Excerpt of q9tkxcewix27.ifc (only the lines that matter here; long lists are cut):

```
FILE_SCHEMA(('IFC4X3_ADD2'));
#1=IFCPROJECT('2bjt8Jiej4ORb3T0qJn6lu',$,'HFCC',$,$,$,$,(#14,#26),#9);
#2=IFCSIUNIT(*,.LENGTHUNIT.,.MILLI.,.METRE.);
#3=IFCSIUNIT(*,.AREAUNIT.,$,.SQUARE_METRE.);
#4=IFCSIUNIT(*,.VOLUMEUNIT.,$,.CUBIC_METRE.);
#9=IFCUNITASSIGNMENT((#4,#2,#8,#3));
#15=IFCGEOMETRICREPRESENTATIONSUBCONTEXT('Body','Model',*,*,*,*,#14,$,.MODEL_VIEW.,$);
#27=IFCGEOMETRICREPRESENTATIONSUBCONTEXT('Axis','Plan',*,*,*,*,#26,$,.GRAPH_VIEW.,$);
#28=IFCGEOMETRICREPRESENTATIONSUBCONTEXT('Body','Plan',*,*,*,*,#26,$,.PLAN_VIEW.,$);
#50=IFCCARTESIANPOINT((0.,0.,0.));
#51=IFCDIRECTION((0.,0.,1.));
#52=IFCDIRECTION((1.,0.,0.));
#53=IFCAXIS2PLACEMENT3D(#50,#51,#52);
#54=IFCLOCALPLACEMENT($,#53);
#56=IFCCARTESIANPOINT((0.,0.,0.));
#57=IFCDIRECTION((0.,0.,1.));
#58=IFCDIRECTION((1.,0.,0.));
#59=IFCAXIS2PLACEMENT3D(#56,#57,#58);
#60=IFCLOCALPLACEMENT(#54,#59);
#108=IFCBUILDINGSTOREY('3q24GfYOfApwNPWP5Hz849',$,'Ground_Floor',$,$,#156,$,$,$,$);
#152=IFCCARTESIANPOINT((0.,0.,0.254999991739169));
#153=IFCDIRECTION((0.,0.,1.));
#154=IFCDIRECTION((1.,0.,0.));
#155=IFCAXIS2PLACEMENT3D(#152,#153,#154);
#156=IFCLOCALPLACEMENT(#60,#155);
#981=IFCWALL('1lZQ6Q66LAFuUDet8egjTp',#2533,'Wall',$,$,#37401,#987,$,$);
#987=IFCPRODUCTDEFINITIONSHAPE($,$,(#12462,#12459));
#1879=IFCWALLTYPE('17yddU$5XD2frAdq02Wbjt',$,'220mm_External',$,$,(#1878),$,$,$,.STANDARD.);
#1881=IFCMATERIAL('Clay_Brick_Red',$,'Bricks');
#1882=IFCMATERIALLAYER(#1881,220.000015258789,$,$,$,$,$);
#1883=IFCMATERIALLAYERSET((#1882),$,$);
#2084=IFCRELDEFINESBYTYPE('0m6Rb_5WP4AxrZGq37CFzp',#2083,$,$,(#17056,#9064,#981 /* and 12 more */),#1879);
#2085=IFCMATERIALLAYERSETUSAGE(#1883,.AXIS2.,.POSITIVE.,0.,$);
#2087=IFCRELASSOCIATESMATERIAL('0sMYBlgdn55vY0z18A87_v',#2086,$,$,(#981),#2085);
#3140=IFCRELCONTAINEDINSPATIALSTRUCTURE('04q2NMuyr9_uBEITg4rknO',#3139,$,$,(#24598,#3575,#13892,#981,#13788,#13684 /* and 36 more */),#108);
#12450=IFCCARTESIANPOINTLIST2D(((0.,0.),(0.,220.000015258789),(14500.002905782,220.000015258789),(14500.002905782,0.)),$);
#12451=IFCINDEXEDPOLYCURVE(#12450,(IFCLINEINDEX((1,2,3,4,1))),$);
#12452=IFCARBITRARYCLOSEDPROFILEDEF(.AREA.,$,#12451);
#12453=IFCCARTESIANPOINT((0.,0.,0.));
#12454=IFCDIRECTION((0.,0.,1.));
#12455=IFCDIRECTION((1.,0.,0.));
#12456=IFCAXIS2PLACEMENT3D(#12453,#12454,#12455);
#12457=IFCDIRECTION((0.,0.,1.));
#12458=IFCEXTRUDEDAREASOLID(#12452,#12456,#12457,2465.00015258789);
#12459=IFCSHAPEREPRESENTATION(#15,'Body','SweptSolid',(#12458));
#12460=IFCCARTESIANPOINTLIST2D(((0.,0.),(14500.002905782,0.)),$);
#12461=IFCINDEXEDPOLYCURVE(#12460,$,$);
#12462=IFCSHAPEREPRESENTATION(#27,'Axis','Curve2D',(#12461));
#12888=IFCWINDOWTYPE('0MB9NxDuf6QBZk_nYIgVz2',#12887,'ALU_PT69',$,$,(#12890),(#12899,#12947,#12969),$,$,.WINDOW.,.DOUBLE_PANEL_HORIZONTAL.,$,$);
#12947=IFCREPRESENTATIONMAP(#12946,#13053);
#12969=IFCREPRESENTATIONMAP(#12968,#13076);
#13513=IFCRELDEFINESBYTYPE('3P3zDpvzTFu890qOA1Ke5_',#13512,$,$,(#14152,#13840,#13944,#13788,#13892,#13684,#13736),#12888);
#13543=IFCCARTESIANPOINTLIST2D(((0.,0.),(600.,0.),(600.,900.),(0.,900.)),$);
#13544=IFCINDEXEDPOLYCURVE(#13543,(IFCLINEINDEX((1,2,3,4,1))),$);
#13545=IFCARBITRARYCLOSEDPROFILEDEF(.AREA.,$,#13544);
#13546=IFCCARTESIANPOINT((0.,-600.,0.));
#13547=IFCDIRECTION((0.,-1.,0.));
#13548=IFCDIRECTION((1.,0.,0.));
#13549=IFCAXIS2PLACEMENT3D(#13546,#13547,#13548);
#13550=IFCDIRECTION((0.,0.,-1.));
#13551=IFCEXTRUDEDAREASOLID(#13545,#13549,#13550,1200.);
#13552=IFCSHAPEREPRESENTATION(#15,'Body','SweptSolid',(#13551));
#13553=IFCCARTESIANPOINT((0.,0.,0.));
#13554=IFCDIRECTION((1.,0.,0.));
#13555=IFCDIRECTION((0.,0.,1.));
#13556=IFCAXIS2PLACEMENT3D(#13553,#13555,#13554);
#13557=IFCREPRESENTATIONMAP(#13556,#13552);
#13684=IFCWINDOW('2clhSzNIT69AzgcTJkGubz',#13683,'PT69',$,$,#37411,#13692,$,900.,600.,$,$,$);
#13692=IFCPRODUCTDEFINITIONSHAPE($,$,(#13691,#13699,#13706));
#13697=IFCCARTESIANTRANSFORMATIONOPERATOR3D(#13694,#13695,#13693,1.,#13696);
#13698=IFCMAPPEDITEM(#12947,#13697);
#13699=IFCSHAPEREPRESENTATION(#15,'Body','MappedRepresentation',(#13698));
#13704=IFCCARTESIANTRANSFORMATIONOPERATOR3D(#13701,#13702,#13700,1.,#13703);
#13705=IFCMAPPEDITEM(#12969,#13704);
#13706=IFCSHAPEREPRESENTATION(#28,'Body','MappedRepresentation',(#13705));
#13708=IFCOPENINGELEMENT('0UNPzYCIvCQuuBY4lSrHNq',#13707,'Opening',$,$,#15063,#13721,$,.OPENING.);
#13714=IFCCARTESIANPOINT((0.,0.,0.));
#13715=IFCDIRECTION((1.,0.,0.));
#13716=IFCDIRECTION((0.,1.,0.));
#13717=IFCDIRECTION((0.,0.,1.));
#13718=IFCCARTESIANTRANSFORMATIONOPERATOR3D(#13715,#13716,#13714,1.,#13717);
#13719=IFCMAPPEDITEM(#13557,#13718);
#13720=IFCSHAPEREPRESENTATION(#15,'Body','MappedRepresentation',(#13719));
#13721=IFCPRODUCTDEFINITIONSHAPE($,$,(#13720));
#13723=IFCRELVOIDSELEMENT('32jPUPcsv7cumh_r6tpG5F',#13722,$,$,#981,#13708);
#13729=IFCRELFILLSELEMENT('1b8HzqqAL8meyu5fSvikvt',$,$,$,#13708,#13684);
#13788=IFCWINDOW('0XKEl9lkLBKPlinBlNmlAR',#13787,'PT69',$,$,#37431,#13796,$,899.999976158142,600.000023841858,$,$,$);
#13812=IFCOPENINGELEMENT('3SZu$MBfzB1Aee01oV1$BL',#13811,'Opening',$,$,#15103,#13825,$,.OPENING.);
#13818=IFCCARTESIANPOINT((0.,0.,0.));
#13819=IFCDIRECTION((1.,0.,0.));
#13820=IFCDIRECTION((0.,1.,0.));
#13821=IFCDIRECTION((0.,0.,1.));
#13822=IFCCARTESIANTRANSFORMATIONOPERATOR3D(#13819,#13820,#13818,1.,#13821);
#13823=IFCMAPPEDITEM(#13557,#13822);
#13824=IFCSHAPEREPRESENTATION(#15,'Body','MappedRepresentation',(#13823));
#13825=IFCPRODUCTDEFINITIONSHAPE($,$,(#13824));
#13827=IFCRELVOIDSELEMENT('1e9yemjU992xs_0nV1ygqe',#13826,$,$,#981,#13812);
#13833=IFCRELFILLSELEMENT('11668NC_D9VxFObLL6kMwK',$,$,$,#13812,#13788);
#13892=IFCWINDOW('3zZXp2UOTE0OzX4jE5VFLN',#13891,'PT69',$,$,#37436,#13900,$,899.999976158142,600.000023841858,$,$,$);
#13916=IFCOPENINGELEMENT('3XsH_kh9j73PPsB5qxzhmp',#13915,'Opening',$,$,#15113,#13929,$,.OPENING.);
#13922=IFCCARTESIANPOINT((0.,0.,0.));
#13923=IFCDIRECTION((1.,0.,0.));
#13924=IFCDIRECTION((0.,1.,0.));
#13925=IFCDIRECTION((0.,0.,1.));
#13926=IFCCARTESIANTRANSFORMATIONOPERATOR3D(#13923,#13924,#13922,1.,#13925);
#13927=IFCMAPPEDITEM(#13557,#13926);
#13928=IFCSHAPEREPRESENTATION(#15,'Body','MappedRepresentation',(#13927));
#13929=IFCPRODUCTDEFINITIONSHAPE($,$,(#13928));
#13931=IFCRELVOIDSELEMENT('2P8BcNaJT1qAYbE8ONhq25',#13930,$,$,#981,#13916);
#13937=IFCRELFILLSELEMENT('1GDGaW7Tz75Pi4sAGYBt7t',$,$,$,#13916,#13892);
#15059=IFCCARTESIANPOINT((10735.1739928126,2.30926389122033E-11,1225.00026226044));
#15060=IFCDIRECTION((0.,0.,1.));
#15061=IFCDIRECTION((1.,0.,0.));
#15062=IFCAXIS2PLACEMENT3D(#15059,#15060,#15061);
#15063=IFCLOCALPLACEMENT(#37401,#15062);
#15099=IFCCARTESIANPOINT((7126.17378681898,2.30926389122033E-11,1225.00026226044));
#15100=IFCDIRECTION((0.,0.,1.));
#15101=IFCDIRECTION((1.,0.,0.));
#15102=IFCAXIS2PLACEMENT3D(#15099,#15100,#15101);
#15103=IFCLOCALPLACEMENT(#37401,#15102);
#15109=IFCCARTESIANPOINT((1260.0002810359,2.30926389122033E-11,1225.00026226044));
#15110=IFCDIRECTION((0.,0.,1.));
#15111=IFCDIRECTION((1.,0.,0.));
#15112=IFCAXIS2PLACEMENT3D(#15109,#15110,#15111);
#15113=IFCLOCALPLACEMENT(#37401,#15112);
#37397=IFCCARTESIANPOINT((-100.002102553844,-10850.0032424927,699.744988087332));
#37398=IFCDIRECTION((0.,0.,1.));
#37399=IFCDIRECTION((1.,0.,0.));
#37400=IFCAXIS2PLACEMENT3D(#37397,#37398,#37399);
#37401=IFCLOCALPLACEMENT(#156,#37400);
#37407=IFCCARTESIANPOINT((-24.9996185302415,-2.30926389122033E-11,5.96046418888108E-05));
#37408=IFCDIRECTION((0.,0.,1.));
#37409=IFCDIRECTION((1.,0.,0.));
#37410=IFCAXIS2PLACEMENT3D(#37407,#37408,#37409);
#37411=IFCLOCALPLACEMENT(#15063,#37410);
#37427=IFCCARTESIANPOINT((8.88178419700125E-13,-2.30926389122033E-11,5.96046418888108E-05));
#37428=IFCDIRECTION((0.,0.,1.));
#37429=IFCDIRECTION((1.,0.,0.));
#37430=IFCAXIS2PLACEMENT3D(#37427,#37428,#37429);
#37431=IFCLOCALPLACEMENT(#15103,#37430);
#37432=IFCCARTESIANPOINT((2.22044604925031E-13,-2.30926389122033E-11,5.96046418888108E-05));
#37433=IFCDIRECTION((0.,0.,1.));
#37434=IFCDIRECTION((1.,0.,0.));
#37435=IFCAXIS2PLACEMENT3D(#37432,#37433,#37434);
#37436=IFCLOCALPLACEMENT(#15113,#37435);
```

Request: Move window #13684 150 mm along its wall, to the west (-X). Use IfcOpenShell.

```python
import ifcopenshell
import ifcopenshell.api.geometry
import ifcopenshell.util.placement
import ifcopenshell.util.unit

model = ifcopenshell.open("q9tkxcewix27.ifc")
unit_scale = ifcopenshell.util.unit.calculate_unit_scale(model)

window = model.by_guid("2clhSzNIT69AzgcTJkGubz")
opening = window.FillsVoids[0].RelatingOpeningElement
wall = opening.VoidsElements[0].RelatingBuildingElement

wall_matrix = ifcopenshell.util.placement.get_local_placement(wall.ObjectPlacement)
shift = wall_matrix[:3, 0] * -0.15 / unit_scale
before = ifcopenshell.util.placement.get_local_placement(window.ObjectPlacement)[:3, 3].copy()

# The window is placed relative to its opening, so it follows when the opening moves.
matrix = ifcopenshell.util.placement.get_local_placement(opening.ObjectPlacement)
matrix[:3, 3] += shift
ifcopenshell.api.geometry.edit_object_placement(
    model, product=opening, matrix=matrix, is_si=False, should_transform_children=True
)

after = ifcopenshell.util.placement.get_local_placement(window.ObjectPlacement)[:3, 3]
print("window moved by", (after - before).round(3) + 0.0)

model.write("q9tkxcewix27_edited.ifc")
```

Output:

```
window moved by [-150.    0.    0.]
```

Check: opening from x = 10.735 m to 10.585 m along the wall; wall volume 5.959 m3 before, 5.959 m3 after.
